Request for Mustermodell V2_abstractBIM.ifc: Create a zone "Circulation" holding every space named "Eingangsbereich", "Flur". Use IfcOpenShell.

First a look at what the model holds.

```python
import ifcopenshell

model = ifcopenshell.open("Mustermodell V2_abstractBIM.ifc")
print(model.schema)
seen = {}
for space in model.by_type("IfcSpace"):
    seen[space.LongName] = seen.get(space.LongName, 0) + 1
for name, count in sorted(seen.items(), key=str):
    print(count, "x", name)
print("zones:", [z.Name for z in model.by_type("IfcZone")][:20])
```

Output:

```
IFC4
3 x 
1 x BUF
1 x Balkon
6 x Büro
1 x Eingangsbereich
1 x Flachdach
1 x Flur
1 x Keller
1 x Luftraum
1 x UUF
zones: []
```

```python
import ifcopenshell
import ifcopenshell.api.group
import ifcopenshell.api.root

model = ifcopenshell.open("Mustermodell V2_abstractBIM.ifc")

names = {"Eingangsbereich", "Flur"}
spaces = [s for s in model.by_type("IfcSpace") if s.LongName in names]

zone = ifcopenshell.api.root.create_entity(model, ifc_class="IfcZone", name="Circulation")
ifcopenshell.api.group.assign_group(model, products=spaces, group=zone)
print(len(spaces), "spaces in", zone.Name)

model.write("Mustermodell V2_abstractBIM_updated.ifc")
```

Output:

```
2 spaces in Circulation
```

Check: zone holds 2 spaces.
